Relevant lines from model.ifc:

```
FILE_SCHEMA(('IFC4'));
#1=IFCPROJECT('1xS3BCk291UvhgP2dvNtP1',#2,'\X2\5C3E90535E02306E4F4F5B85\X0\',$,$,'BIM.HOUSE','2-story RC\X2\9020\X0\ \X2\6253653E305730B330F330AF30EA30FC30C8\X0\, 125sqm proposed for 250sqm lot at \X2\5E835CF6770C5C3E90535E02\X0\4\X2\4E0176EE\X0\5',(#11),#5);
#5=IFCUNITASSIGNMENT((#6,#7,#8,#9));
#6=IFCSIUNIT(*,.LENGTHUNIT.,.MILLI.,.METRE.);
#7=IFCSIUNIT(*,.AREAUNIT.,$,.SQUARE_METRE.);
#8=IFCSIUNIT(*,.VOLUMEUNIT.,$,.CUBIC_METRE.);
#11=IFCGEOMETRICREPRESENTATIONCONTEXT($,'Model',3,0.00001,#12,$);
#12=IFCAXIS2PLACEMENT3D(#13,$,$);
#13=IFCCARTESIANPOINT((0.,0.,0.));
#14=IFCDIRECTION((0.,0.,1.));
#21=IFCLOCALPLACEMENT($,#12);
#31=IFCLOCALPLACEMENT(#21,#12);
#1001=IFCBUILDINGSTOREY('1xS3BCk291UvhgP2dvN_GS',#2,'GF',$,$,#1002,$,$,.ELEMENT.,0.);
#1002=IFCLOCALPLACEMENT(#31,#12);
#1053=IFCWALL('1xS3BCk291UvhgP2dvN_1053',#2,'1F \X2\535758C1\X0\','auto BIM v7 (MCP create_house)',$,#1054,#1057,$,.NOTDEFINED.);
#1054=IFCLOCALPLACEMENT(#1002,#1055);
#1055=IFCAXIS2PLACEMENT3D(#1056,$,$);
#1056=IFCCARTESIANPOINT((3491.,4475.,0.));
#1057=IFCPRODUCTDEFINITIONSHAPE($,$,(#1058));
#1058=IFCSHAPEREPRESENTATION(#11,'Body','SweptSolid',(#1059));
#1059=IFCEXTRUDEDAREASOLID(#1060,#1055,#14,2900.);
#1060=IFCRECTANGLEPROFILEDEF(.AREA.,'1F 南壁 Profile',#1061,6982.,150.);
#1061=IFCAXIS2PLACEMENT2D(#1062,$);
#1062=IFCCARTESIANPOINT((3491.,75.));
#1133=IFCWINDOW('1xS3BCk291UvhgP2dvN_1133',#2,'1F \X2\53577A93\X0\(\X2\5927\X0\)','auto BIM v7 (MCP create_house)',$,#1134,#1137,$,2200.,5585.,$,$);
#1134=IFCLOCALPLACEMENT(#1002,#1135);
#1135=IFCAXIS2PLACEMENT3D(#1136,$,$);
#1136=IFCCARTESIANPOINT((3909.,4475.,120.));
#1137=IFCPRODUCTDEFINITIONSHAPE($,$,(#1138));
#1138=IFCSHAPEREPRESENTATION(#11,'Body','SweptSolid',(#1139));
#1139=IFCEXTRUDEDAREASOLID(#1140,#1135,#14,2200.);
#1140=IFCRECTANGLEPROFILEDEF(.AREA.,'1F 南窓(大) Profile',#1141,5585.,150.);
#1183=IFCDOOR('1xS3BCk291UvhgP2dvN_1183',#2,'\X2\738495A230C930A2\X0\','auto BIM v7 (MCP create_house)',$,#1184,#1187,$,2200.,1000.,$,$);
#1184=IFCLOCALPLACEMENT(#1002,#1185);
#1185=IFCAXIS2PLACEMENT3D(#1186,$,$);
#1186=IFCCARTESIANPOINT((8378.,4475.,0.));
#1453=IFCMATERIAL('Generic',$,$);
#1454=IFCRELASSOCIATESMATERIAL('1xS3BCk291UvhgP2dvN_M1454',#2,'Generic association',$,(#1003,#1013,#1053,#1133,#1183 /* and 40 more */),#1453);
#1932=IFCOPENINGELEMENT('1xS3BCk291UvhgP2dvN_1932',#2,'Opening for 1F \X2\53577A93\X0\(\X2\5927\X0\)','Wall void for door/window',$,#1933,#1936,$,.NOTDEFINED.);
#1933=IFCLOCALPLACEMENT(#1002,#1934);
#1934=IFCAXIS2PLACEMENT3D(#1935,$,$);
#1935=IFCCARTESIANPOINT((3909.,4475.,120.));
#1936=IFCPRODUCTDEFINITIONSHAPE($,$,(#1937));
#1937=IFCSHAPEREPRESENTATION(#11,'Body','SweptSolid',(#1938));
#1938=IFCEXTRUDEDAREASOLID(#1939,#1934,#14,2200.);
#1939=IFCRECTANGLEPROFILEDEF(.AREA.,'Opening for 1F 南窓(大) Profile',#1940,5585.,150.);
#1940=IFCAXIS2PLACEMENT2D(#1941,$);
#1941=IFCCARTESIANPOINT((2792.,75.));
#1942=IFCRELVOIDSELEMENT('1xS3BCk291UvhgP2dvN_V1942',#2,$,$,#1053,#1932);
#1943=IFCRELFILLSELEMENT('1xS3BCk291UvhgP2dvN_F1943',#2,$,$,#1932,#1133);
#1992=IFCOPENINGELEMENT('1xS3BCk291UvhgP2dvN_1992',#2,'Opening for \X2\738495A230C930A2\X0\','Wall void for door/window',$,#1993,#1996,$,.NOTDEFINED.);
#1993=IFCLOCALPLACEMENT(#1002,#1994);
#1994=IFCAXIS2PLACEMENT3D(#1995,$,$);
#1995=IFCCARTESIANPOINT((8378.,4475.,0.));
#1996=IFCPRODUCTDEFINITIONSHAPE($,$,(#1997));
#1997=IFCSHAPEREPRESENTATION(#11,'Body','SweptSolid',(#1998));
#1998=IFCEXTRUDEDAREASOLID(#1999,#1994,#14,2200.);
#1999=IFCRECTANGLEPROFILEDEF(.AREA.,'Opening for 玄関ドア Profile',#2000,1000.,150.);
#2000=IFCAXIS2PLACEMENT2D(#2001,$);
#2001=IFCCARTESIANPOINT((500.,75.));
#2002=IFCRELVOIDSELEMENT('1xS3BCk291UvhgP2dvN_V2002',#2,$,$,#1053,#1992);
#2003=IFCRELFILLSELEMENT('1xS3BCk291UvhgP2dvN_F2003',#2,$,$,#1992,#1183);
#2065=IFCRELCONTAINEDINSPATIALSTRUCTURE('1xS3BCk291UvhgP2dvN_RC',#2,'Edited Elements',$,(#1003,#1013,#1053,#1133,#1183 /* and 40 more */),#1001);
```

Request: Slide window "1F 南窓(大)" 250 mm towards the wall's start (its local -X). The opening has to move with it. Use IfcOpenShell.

```python
import ifcopenshell
import ifcopenshell.api.geometry
import ifcopenshell.util.placement
import ifcopenshell.util.unit

model = ifcopenshell.open("model.ifc")
unit_scale = ifcopenshell.util.unit.calculate_unit_scale(model)

window = model.by_id(1133)
opening = window.FillsVoids[0].RelatingOpeningElement
wall = opening.VoidsElements[0].RelatingBuildingElement

wall_matrix = ifcopenshell.util.placement.get_local_placement(wall.ObjectPlacement)
shift = wall_matrix[:3, 0] * -0.25 / unit_scale
before = ifcopenshell.util.placement.get_local_placement(window.ObjectPlacement)[:3, 3].copy()

# The window is not placed relative to its opening, so move both.
for product in (opening, window):
    matrix = ifcopenshell.util.placement.get_local_placement(product.ObjectPlacement)
    matrix[:3, 3] += shift
    ifcopenshell.api.geometry.edit_object_placement(model, product=product, matrix=matrix, is_si=False)

after = ifcopenshell.util.placement.get_local_placement(window.ObjectPlacement)[:3, 3]
print("window moved by", (after - before).round(3) + 0.0)

model.write("model_updated.ifc")
```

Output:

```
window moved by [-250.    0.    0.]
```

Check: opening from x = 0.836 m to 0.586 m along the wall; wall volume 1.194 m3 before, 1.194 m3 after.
